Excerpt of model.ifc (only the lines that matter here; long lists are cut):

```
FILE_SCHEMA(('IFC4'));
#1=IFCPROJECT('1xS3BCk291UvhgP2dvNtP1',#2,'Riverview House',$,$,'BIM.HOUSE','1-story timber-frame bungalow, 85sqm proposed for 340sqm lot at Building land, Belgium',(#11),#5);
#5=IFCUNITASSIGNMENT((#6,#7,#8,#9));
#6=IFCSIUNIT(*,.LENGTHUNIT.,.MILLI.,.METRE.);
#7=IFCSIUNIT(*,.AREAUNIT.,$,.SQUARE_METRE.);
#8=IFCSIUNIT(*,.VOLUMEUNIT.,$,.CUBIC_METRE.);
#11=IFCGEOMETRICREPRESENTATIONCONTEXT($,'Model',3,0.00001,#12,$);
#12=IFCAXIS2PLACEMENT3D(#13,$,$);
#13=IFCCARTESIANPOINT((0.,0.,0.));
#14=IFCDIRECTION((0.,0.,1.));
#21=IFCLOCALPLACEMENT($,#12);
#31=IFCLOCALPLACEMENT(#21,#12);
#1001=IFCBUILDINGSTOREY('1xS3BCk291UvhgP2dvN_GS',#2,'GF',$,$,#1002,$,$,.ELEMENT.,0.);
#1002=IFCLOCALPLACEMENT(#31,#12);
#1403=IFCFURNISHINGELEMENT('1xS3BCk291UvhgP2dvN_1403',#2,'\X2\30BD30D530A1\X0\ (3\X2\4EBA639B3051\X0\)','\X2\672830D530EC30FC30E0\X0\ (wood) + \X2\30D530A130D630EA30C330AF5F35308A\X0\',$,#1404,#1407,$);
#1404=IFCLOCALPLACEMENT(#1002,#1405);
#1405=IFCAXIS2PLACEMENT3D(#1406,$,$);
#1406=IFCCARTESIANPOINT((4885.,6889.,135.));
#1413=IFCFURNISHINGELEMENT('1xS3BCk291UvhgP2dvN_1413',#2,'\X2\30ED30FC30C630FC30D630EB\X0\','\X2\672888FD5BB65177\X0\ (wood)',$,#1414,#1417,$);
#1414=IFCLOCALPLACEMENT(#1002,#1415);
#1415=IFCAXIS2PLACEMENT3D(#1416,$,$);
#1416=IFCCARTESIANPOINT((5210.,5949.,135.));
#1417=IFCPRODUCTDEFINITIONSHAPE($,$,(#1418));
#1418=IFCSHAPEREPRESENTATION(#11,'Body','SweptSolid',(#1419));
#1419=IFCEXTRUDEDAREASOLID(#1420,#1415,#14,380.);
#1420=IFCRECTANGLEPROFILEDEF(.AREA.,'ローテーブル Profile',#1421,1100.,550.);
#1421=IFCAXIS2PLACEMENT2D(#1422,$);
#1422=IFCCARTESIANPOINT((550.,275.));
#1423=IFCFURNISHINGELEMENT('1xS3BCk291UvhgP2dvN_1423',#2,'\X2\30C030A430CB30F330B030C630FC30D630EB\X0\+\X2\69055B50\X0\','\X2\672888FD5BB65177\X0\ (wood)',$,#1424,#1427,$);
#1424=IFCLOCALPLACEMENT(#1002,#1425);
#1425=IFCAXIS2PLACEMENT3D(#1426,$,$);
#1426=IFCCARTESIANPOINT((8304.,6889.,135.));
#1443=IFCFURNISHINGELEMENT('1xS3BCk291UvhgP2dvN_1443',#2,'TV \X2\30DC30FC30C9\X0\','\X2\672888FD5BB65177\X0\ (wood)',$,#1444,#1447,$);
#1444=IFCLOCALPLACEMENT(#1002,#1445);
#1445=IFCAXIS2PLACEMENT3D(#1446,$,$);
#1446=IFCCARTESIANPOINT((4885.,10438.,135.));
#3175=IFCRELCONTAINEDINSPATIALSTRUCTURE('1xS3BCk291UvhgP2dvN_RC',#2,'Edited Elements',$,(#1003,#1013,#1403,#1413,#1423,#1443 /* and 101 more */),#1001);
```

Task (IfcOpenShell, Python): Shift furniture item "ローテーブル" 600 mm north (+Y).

```python
import ifcopenshell
import ifcopenshell.api.geometry
import ifcopenshell.util.placement
import ifcopenshell.util.unit

model = ifcopenshell.open("model.ifc")
unit_scale = ifcopenshell.util.unit.calculate_unit_scale(model)

item = model.by_guid("1xS3BCk291UvhgP2dvN_1413")
matrix = ifcopenshell.util.placement.get_local_placement(item.ObjectPlacement)
matrix[1, 3] += 0.6 / unit_scale
ifcopenshell.api.geometry.edit_object_placement(model, product=item, matrix=matrix, is_si=False)

print(ifcopenshell.util.placement.get_local_placement(item.ObjectPlacement).round(3) + 0.0)

model.write("model_edited.ifc")
```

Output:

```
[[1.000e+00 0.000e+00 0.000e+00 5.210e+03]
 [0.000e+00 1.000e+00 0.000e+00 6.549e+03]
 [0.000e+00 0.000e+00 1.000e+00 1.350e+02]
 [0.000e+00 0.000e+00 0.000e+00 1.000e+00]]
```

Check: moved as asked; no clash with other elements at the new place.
